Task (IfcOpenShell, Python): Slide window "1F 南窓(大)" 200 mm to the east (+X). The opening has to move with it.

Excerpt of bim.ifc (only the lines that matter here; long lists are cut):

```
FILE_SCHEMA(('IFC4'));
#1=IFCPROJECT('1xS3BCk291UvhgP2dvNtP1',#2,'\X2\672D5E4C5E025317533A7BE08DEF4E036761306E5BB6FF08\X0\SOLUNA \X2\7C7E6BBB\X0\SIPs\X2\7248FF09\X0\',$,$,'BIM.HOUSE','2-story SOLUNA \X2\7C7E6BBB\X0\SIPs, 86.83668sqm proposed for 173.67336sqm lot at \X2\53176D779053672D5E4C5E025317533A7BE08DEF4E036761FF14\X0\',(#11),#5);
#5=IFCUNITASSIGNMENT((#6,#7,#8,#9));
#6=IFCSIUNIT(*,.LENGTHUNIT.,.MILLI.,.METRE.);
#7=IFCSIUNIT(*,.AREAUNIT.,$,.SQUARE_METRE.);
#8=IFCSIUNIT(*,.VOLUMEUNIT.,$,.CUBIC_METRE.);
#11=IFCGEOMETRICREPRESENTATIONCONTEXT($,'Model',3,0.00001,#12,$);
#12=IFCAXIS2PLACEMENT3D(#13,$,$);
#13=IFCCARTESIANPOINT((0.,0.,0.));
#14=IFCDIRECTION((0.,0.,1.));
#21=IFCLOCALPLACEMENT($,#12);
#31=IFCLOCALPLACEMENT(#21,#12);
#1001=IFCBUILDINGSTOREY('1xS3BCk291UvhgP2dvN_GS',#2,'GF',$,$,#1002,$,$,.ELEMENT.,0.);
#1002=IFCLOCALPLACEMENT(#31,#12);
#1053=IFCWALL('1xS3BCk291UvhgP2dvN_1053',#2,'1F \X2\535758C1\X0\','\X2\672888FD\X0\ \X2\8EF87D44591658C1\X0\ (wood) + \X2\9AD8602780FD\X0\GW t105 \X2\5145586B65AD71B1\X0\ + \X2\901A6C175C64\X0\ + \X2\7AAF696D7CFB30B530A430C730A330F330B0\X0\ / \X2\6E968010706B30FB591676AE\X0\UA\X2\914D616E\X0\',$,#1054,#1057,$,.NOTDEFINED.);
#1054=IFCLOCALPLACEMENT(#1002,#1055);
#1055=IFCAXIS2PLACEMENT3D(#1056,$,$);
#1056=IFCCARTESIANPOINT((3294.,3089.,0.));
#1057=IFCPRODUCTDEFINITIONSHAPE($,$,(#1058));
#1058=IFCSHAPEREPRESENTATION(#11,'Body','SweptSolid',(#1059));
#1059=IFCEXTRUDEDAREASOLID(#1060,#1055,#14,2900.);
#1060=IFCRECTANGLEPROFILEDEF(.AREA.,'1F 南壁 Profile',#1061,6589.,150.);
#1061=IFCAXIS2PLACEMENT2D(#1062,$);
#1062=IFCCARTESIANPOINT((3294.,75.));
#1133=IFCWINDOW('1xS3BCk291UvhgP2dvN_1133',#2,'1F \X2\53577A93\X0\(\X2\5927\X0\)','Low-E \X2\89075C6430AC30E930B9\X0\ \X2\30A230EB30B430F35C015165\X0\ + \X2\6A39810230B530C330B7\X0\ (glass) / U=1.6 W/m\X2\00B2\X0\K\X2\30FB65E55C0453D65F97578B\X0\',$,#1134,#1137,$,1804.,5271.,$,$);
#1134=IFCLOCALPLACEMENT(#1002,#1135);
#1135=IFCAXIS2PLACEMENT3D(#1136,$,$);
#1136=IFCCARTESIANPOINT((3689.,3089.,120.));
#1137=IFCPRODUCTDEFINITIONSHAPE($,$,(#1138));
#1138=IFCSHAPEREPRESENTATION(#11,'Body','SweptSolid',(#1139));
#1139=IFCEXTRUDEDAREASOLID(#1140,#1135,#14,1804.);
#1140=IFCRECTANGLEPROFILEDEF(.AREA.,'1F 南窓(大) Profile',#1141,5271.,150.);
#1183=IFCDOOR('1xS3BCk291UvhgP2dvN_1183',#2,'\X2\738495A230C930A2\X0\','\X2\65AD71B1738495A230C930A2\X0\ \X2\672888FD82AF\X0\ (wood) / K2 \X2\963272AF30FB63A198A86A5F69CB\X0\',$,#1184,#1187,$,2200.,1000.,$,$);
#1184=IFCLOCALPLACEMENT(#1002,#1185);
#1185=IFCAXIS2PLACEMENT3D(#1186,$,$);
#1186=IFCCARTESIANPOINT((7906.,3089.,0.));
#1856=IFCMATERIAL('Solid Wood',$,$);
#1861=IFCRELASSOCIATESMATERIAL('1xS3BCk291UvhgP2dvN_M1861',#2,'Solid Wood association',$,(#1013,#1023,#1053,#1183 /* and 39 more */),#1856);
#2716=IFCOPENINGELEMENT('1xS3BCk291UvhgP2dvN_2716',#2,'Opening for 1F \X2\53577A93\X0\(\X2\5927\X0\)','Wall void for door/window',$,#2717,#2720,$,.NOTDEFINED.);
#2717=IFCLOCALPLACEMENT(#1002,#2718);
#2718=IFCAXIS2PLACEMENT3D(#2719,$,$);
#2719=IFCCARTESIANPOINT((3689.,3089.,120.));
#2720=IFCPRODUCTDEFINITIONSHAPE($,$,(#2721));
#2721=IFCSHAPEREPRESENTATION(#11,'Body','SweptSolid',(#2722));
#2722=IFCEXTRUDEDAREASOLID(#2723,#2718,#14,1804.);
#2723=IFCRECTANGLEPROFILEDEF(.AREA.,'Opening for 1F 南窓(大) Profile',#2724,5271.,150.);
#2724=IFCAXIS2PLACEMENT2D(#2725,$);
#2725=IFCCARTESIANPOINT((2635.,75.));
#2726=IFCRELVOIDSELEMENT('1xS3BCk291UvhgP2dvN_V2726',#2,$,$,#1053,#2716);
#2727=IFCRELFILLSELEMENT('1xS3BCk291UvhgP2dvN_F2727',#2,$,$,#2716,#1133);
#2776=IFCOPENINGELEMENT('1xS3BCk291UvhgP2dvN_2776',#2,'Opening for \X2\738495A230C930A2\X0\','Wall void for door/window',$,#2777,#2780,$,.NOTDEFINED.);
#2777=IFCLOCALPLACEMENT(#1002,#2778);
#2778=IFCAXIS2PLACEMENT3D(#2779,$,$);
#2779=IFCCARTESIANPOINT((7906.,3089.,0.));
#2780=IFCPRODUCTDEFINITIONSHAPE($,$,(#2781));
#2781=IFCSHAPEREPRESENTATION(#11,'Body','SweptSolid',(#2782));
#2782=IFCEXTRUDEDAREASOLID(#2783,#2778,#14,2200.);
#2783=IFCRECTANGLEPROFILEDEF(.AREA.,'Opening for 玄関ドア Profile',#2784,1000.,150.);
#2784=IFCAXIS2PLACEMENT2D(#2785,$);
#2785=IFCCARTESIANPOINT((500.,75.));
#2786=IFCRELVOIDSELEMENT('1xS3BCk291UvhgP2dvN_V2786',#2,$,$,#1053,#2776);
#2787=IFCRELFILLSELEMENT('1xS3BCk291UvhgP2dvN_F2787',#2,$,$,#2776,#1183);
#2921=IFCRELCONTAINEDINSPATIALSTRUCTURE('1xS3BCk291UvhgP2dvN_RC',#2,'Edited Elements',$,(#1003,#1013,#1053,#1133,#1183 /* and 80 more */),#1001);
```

```python
import ifcopenshell
import ifcopenshell.api.geometry
import ifcopenshell.util.placement
import ifcopenshell.util.unit

model = ifcopenshell.open("bim.ifc")
unit_scale = ifcopenshell.util.unit.calculate_unit_scale(model)

window = model.by_guid("1xS3BCk291UvhgP2dvN_1133")
opening = window.FillsVoids[0].RelatingOpeningElement
wall = opening.VoidsElements[0].RelatingBuildingElement

wall_matrix = ifcopenshell.util.placement.get_local_placement(wall.ObjectPlacement)
shift = wall_matrix[:3, 0] * 0.2 / unit_scale
before = ifcopenshell.util.placement.get_local_placement(window.ObjectPlacement)[:3, 3].copy()

# The window is not placed relative to its opening, so move both.
for product in (opening, window):
    matrix = ifcopenshell.util.placement.get_local_placement(product.ObjectPlacement)
    matrix[:3, 3] += shift
    ifcopenshell.api.geometry.edit_object_placement(model, product=product, matrix=matrix, is_si=False)

after = ifcopenshell.util.placement.get_local_placement(window.ObjectPlacement)[:3, 3]
print("window moved by", (after - before).round(3) + 0.0)

model.write("bim_v2.ifc")
```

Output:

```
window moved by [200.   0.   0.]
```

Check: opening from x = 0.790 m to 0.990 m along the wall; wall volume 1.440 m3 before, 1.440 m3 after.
